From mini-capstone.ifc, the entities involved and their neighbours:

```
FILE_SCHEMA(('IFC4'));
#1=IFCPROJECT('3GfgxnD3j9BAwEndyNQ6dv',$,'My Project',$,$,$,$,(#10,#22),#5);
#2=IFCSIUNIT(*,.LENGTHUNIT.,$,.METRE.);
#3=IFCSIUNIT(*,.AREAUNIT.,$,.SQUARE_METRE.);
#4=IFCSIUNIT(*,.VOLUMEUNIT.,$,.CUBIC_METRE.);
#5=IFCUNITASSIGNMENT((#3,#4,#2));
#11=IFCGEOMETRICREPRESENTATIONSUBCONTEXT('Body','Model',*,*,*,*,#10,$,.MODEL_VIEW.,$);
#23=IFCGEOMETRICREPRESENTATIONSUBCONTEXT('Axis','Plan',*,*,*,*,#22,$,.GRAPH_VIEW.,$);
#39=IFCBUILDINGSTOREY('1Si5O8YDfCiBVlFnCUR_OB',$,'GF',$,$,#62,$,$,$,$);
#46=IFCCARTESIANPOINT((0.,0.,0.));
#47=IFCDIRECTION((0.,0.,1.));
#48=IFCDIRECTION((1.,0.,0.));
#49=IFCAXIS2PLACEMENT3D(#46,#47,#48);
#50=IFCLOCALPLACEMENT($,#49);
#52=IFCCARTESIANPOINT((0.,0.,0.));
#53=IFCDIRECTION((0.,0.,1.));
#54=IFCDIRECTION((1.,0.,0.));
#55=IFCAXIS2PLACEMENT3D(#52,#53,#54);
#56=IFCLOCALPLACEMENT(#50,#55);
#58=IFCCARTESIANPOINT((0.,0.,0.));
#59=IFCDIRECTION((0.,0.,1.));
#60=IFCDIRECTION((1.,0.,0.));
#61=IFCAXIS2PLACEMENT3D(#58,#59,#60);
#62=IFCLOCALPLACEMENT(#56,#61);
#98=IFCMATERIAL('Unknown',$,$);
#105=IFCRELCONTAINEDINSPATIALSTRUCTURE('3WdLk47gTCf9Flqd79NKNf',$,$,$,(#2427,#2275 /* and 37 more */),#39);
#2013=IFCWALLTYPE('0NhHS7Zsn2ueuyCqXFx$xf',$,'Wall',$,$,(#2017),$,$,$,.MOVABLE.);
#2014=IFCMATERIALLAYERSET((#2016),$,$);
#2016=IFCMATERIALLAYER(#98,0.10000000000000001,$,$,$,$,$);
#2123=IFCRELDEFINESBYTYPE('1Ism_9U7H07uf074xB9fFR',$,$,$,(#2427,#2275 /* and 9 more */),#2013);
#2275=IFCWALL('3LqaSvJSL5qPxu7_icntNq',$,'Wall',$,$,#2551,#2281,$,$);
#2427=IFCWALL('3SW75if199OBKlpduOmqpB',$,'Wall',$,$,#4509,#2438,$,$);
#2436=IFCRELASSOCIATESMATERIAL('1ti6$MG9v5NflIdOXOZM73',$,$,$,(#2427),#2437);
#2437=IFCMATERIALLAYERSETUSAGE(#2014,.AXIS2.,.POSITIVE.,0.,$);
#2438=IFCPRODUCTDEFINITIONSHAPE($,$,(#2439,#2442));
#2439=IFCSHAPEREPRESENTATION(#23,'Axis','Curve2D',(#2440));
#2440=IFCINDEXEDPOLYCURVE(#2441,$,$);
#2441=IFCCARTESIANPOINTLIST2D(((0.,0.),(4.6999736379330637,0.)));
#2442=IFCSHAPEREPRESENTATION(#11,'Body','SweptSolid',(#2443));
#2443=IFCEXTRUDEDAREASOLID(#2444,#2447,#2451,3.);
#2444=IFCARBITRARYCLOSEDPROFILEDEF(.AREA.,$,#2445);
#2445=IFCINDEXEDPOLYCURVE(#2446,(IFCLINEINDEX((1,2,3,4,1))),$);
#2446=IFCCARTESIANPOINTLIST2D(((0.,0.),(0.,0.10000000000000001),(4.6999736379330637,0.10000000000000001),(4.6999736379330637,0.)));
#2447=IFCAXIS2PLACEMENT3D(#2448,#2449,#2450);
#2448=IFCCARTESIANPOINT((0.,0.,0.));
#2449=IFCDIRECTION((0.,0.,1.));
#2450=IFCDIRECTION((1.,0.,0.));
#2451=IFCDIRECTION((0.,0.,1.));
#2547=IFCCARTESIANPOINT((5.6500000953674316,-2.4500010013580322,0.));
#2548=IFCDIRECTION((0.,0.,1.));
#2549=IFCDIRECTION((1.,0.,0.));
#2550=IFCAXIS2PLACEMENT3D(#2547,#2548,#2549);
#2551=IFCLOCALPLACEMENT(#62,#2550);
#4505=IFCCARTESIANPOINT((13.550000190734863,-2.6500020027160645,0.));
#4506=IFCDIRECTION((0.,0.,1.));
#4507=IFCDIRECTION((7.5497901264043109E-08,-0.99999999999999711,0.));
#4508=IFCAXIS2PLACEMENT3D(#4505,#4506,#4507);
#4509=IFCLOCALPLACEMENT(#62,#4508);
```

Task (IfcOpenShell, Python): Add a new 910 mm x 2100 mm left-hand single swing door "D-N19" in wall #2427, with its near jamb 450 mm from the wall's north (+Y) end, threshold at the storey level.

```python
import numpy as np
import ifcopenshell
import ifcopenshell.api.feature
import ifcopenshell.api.geometry
import ifcopenshell.api.root
import ifcopenshell.api.spatial
import ifcopenshell.geom
import ifcopenshell.util.element
import ifcopenshell.util.placement
import ifcopenshell.util.representation
import ifcopenshell.util.shape
import ifcopenshell.util.unit

model = ifcopenshell.open("mini-capstone.ifc")
unit_scale = ifcopenshell.util.unit.calculate_unit_scale(model)
settings = ifcopenshell.geom.settings()


def volume(element):
    """Net volume in cubic metres, openings subtracted."""
    shape = ifcopenshell.geom.create_shape(settings, element)
    return ifcopenshell.util.shape.get_volume(shape.geometry)


wall = model.by_guid("3SW75if199OBKlpduOmqpB")
storey = ifcopenshell.util.element.get_container(wall, ifc_class="IfcBuildingStorey")
context = ifcopenshell.util.representation.get_context(model, "Model", "Body", "MODEL_VIEW")
before = volume(wall)

width, height, from_end, sill = 0.91, 2.1, 0.45, 0.0  # metres

# The wall runs along its own X axis, and the end named is its -X end.
wall_shape = ifcopenshell.geom.create_shape(settings, wall)
x, y, z = ifcopenshell.util.shape.get_vertices(wall_shape.geometry).T
start = x.min() + from_end
face, thickness = float(y.min()), float(y.max() - y.min())
wall_matrix = ifcopenshell.util.placement.get_local_placement(wall.ObjectPlacement)
level = ifcopenshell.util.placement.get_local_placement(storey.ObjectPlacement)[2, 3]


def in_wall(x, y):
    """Placement at x, y metres in the wall's axes, at sill height."""
    matrix = wall_matrix.copy()
    matrix[:, 3] = wall_matrix @ np.array([x / unit_scale, y / unit_scale, 0.0, 1.0])
    matrix[2, 3] = level + sill / unit_scale
    return matrix


# Opening: a box that overshoots both wall faces by 50 mm.
opening = ifcopenshell.api.root.create_entity(model, ifc_class="IfcOpeningElement", predefined_type="OPENING")
box = ifcopenshell.api.geometry.add_wall_representation(
    model, context=context, length=width, height=height, thickness=thickness + 0.1
)
ifcopenshell.api.geometry.assign_representation(model, product=opening, representation=box)
ifcopenshell.api.geometry.edit_object_placement(model, product=opening, matrix=in_wall(start, face - 0.05), is_si=False)
ifcopenshell.api.feature.add_feature(model, feature=opening, element=wall)

door = ifcopenshell.api.root.create_entity(model, ifc_class="IfcDoor", name="D-N19", predefined_type="DOOR")
door.OverallWidth, door.OverallHeight = width / unit_scale, height / unit_scale
door.OperationType = "SINGLE_SWING_LEFT"
body = ifcopenshell.api.geometry.add_door_representation(
    model,
    context=context,
    overall_width=door.OverallWidth,
    overall_height=door.OverallHeight,
    operation_type="SINGLE_SWING_LEFT",
    lining_properties={"LiningDepth": thickness / unit_scale, "ThresholdDepth": thickness / unit_scale},
)
ifcopenshell.api.geometry.assign_representation(model, product=door, representation=body)
ifcopenshell.api.spatial.assign_container(model, products=[door], relating_structure=storey)
ifcopenshell.api.feature.add_filling(model, opening=opening, element=door)

# The lining spans the wall, so the door starts at the wall face.
ifcopenshell.api.geometry.edit_object_placement(model, product=door, matrix=in_wall(start, face), is_si=False)

after = volume(wall)

print(f"wall volume {before:.3f} -> {after:.3f} m3")

model.write("mini-capstone-out.ifc")
```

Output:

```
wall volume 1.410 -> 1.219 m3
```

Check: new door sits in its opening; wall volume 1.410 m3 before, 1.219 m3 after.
